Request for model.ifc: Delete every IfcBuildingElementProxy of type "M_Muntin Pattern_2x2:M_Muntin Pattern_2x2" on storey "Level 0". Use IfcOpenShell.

First a look at what the model holds.

```python
import ifcopenshell
import ifcopenshell.util.element

model = ifcopenshell.open("model.ifc")
print(model.schema)
storey = next(s for s in model.by_type("IfcBuildingStorey") if s.Name == "Level 0")
proxies = [e for e in ifcopenshell.util.element.get_decomposition(storey) if e.is_a("IfcBuildingElementProxy")]
seen = {}
for e in proxies:
    element_type = ifcopenshell.util.element.get_type(e)
    name = element_type.Name if element_type not in (None, e) else None
    seen[name] = seen.get(name, 0) + 1
for name, count in sorted(seen.items(), key=str):
    print(count, "x", name)
```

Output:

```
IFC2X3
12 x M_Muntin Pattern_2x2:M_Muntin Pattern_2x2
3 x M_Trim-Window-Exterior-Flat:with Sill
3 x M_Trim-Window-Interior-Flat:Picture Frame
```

```python
import ifcopenshell
import ifcopenshell.api.root
import ifcopenshell.util.element

model = ifcopenshell.open("model.ifc")

storey = next(s for s in model.by_type("IfcBuildingStorey") if s.Name == "Level 0")
proxies = [e for e in ifcopenshell.util.element.get_decomposition(storey) if e.is_a("IfcBuildingElementProxy")]
targets = [e for e in proxies if (t := ifcopenshell.util.element.get_type(e)) not in (None, e) and t.Name == "M_Muntin Pattern_2x2:M_Muntin Pattern_2x2"]

for e in targets:
    ifcopenshell.api.root.remove_product(model, product=e)
print(len(targets), "removed")

model.write("model_updated.ifc")
```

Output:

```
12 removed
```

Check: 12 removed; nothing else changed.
